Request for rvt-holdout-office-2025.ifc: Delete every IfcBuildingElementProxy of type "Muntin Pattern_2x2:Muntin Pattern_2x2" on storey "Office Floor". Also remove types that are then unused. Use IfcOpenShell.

First a look at what the model holds.

```python
import ifcopenshell
import ifcopenshell.util.element

model = ifcopenshell.open("rvt-holdout-office-2025.ifc")
print(model.schema)
storey = next(s for s in model.by_type("IfcBuildingStorey") if s.Name == "Office Floor")
proxies = [e for e in ifcopenshell.util.element.get_decomposition(storey) if e.is_a("IfcBuildingElementProxy")]
seen = {}
for e in proxies:
    element_type = ifcopenshell.util.element.get_type(e)
    name = element_type.Name if element_type not in (None, e) else None
    seen[name] = seen.get(name, 0) + 1
for name, count in sorted(seen.items(), key=str):
    print(count, "x", name)
```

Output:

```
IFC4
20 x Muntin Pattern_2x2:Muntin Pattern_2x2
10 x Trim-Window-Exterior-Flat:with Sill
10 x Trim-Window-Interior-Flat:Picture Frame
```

```python
import ifcopenshell
import ifcopenshell.api.root
import ifcopenshell.util.element

model = ifcopenshell.open("rvt-holdout-office-2025.ifc")

storey = next(s for s in model.by_type("IfcBuildingStorey") if s.Name == "Office Floor")
proxies = [e for e in ifcopenshell.util.element.get_decomposition(storey) if e.is_a("IfcBuildingElementProxy")]
targets = [e for e in proxies if (t := ifcopenshell.util.element.get_type(e)) not in (None, e) and t.Name == "Muntin Pattern_2x2:Muntin Pattern_2x2"]
types = {ifcopenshell.util.element.get_type(e) for e in targets} - {None, *targets}

for e in targets:
    ifcopenshell.api.root.remove_product(model, product=e)
print(len(targets), "removed")

unused = [t for t in types if not ifcopenshell.util.element.get_types(t)]
for t in unused:
    ifcopenshell.api.root.remove_product(model, product=t)
print(len(unused), "unused types removed")

model.write("rvt-holdout-office-2025_edited.ifc")
```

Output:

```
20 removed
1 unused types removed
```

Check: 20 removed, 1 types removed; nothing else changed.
